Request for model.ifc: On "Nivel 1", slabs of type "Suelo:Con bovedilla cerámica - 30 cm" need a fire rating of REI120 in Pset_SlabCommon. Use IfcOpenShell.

First a look at what the model holds.

```python
import ifcopenshell
import ifcopenshell.util.element

model = ifcopenshell.open("model.ifc")
print(model.schema)
storey = next(s for s in model.by_type("IfcBuildingStorey") if s.Name == "Nivel 1")
slabs = [e for e in ifcopenshell.util.element.get_decomposition(storey) if e.is_a("IfcSlab")]
seen = {}
for e in slabs:
    element_type = ifcopenshell.util.element.get_type(e)
    key = (element_type.Name if element_type != e and element_type else None, ifcopenshell.util.element.get_pset(e, "Pset_SlabCommon", "FireRating"))
    seen[key] = seen.get(key, 0) + 1
for (name, value), count in sorted(seen.items(), key=str):
    print(count, "x", name, "|", value)
```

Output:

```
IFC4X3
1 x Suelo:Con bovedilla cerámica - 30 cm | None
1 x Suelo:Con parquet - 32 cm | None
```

```python
import ifcopenshell
import ifcopenshell.api.pset
import ifcopenshell.util.element

model = ifcopenshell.open("model.ifc")

storey = next(s for s in model.by_type("IfcBuildingStorey") if s.Name == "Nivel 1")
slabs = [e for e in ifcopenshell.util.element.get_decomposition(storey) if e.is_a("IfcSlab")]

count = 0
for e in slabs:
    element_type = ifcopenshell.util.element.get_type(e)
    if element_type in (None, e) or element_type.Name != "Suelo:Con bovedilla cerámica - 30 cm":
        continue
    # add_pset returns the element's existing set when there is one.
    pset = ifcopenshell.api.pset.add_pset(model, product=e, name="Pset_SlabCommon")
    ifcopenshell.api.pset.edit_pset(model, pset=pset, properties={"FireRating": "REI120"})
    count += 1

print(count, "slabs updated")

model.write("model-out.ifc")
```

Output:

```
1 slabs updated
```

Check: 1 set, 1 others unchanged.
